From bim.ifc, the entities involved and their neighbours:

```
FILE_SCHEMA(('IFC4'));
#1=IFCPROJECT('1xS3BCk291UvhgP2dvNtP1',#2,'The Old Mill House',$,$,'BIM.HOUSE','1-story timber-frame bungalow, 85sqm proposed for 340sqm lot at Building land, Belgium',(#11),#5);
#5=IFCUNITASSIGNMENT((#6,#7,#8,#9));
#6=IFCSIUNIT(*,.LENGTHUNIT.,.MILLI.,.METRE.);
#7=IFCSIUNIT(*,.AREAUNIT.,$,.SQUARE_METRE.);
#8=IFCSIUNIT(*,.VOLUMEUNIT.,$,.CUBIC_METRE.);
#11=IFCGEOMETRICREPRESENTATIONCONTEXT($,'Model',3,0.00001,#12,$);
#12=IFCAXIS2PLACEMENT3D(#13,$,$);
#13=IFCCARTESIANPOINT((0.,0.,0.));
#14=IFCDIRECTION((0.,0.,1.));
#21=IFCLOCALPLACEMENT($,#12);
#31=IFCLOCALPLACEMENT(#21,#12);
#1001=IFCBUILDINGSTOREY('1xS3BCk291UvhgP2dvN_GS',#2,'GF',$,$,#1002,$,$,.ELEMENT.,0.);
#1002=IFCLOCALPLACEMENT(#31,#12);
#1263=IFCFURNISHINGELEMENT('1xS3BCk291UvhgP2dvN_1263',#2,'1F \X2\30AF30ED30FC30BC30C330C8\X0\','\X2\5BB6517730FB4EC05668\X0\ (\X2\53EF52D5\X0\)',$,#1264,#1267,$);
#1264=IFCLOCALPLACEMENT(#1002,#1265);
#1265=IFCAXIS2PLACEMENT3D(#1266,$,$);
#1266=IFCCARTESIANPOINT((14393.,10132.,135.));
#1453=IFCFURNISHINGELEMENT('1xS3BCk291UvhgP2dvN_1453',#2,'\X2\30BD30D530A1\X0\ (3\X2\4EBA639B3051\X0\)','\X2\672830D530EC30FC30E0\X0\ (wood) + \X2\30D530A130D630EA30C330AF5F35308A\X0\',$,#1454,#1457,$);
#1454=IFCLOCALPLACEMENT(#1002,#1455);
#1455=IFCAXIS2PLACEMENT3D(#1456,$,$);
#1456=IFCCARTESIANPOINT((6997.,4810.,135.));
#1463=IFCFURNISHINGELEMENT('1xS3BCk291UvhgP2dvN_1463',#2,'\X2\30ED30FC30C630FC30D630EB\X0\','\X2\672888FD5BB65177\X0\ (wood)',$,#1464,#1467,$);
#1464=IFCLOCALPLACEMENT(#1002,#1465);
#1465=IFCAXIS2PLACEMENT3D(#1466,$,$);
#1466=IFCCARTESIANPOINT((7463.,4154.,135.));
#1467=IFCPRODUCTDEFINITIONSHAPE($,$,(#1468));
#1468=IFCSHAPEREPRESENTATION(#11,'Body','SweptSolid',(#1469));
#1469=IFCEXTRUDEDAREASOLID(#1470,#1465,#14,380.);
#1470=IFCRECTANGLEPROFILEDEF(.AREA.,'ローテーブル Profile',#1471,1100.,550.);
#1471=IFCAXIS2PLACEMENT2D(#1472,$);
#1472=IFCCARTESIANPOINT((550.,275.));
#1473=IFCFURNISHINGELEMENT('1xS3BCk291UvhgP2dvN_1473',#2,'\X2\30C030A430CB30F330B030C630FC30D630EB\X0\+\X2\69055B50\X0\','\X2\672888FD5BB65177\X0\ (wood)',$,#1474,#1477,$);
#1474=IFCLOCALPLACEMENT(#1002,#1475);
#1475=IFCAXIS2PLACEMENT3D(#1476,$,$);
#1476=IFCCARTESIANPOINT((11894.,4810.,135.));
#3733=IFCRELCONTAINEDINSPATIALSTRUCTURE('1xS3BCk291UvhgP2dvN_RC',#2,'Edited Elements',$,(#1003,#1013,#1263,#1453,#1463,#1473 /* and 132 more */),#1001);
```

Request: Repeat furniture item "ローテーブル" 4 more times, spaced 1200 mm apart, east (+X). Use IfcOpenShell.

```python
import numpy as np
import ifcopenshell
import ifcopenshell.api.geometry
import ifcopenshell.api.root
import ifcopenshell.util.element
import ifcopenshell.util.placement

model = ifcopenshell.open("bim.ifc")


def reuse_history(source, copy):
    """copy_class also copies each property set's owner history, people and application; keep the originals."""
    for rel in copy.IsDefinedBy:
        if rel.is_a("IfcRelDefinesByProperties") and (history := rel.RelatingPropertyDefinition.OwnerHistory):
            rel.RelatingPropertyDefinition.OwnerHistory = source.OwnerHistory
            ifcopenshell.util.element.remove_deep2(model, history)


source = model.by_guid("1xS3BCk291UvhgP2dvN_1463")
base = ifcopenshell.util.placement.get_local_placement(source.ObjectPlacement)
step = np.array([1.0, 0.0, 0.0]) * 1200.0

for i in range(1, 5):
    copy = ifcopenshell.api.root.copy_class(model, product=source)
    copy.Representation = ifcopenshell.util.element.copy_deep(
        model, source.Representation, exclude=["IfcGeometricRepresentationContext", "IfcRepresentationMap"]
    )
    reuse_history(source, copy)
    matrix = base.copy()
    matrix[:3, 3] += i * step
    print("added at", matrix[:3, 3].round(3) + 0.0)
    ifcopenshell.api.geometry.edit_object_placement(model, product=copy, matrix=matrix, is_si=False)

model.write("bim_rev.ifc")
```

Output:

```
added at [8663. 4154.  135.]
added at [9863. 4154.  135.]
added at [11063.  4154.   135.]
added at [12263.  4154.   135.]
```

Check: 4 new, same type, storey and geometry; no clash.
